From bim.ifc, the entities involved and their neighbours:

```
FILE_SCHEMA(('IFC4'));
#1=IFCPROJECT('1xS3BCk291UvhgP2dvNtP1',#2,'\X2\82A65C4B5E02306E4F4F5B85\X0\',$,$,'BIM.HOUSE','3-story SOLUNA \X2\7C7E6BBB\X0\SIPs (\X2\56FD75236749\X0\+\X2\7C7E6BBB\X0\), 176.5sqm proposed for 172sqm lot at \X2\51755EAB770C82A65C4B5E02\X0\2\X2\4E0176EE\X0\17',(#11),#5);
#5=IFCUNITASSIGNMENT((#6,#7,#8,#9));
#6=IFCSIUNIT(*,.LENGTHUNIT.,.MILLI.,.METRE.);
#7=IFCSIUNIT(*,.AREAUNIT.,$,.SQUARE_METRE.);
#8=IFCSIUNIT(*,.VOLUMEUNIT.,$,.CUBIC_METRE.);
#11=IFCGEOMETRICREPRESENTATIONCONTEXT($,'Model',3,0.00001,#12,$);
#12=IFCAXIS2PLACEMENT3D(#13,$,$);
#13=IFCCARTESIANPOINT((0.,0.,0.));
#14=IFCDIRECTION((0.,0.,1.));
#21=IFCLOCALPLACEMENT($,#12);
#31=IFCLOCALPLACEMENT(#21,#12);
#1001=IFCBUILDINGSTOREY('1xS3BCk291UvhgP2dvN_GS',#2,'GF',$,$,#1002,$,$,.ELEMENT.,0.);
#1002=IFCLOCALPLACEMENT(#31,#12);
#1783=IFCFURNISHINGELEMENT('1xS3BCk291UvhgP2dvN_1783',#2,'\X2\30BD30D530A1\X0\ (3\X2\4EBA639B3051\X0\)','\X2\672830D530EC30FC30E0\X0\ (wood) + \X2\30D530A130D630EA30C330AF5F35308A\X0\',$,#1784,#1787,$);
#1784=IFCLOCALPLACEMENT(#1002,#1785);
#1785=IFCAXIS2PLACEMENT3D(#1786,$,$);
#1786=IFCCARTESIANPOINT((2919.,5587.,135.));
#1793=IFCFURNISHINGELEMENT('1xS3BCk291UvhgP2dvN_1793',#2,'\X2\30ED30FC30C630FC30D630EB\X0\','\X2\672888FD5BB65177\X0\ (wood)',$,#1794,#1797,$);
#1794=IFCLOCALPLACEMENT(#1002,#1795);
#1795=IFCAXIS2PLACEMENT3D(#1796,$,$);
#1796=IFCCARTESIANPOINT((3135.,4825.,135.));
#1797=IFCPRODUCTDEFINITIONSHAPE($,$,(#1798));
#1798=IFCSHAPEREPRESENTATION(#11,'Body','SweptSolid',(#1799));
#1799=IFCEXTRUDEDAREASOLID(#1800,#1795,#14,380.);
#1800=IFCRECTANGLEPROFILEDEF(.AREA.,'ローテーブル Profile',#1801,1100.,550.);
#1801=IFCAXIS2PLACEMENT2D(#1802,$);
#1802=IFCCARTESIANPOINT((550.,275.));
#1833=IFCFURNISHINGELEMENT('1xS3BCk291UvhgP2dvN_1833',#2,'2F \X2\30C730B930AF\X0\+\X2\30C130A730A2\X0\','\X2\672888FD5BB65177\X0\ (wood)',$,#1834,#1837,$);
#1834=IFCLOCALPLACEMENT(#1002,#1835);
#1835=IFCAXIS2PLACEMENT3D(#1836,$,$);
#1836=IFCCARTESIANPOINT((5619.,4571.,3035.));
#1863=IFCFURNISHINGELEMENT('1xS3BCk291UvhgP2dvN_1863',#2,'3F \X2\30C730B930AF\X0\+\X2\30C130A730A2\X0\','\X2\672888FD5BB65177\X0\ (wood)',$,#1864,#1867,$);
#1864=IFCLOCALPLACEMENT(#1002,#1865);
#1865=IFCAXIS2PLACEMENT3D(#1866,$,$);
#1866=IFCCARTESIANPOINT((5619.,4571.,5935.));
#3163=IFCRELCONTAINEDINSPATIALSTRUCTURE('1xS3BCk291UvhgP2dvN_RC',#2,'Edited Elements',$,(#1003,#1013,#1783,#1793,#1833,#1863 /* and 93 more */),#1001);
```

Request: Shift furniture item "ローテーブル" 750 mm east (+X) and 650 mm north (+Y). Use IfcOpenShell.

```python
import ifcopenshell
import ifcopenshell.api.geometry
import ifcopenshell.util.placement
import ifcopenshell.util.unit

model = ifcopenshell.open("bim.ifc")
unit_scale = ifcopenshell.util.unit.calculate_unit_scale(model)

item = model.by_guid("1xS3BCk291UvhgP2dvN_1793")
matrix = ifcopenshell.util.placement.get_local_placement(item.ObjectPlacement)
matrix[0, 3] += 0.75 / unit_scale
matrix[1, 3] += 0.65 / unit_scale
ifcopenshell.api.geometry.edit_object_placement(model, product=item, matrix=matrix, is_si=False)

print(ifcopenshell.util.placement.get_local_placement(item.ObjectPlacement).round(3) + 0.0)

model.write("bim-out.ifc")
```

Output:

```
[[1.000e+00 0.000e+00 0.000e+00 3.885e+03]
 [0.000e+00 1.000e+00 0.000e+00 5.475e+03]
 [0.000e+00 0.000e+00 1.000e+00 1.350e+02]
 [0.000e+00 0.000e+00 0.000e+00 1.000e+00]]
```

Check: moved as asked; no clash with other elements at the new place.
